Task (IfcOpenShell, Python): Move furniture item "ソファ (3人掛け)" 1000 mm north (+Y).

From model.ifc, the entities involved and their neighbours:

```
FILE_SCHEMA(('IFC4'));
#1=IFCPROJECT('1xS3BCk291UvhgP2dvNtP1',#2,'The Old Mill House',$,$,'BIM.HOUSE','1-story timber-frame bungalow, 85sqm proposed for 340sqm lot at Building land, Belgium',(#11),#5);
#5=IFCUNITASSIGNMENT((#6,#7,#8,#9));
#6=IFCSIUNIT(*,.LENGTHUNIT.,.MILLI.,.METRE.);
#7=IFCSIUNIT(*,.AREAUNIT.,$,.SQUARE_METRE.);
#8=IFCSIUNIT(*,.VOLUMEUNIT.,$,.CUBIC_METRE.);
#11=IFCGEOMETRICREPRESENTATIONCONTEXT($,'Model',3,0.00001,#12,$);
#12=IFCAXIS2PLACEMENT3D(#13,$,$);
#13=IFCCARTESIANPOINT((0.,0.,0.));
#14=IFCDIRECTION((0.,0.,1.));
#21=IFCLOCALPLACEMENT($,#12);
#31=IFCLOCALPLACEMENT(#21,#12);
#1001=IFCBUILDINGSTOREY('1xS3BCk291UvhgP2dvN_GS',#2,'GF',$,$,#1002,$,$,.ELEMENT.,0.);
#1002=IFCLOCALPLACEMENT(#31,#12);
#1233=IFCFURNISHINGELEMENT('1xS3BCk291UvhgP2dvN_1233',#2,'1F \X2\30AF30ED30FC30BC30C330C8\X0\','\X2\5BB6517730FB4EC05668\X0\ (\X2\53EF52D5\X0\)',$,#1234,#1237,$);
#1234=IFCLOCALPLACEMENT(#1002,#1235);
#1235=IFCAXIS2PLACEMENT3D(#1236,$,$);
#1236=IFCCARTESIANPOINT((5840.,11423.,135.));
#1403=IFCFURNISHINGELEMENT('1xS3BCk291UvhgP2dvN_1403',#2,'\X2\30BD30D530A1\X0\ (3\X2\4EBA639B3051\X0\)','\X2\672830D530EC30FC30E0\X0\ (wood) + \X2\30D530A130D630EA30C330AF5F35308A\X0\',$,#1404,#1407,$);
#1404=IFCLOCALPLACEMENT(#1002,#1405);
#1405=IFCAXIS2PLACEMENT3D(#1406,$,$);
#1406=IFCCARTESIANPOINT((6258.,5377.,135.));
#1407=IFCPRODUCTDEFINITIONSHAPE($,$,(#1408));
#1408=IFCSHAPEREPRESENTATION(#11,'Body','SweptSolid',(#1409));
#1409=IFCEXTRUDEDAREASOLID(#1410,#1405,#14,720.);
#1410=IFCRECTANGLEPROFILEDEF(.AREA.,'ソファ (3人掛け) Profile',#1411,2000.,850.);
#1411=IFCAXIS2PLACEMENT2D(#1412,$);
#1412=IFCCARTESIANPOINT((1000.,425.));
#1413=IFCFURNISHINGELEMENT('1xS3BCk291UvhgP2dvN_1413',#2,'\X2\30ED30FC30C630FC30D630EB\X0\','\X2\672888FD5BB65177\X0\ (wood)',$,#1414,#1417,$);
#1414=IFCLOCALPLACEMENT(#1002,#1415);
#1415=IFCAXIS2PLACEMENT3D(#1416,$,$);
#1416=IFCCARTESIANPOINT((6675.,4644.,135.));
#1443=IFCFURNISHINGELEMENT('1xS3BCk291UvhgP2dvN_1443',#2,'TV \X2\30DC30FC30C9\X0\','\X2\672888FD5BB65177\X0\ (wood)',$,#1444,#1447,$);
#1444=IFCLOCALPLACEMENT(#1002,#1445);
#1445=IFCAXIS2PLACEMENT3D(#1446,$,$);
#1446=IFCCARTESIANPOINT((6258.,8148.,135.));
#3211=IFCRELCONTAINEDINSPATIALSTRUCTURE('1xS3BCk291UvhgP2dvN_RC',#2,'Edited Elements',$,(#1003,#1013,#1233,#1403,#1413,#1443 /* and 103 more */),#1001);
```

```python
import ifcopenshell
import ifcopenshell.api.geometry
import ifcopenshell.util.placement

model = ifcopenshell.open("model.ifc")

item = model.by_guid("1xS3BCk291UvhgP2dvN_1403")
matrix = ifcopenshell.util.placement.get_local_placement(item.ObjectPlacement)
matrix[1, 3] += 1000.0
ifcopenshell.api.geometry.edit_object_placement(model, product=item, matrix=matrix, is_si=False)

print(ifcopenshell.util.placement.get_local_placement(item.ObjectPlacement).round(3) + 0.0)

model.write("model-out.ifc")
```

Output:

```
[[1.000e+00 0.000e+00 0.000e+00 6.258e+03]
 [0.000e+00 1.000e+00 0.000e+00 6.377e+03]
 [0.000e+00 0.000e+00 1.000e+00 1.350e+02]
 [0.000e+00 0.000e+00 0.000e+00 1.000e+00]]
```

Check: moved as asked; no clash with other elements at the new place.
